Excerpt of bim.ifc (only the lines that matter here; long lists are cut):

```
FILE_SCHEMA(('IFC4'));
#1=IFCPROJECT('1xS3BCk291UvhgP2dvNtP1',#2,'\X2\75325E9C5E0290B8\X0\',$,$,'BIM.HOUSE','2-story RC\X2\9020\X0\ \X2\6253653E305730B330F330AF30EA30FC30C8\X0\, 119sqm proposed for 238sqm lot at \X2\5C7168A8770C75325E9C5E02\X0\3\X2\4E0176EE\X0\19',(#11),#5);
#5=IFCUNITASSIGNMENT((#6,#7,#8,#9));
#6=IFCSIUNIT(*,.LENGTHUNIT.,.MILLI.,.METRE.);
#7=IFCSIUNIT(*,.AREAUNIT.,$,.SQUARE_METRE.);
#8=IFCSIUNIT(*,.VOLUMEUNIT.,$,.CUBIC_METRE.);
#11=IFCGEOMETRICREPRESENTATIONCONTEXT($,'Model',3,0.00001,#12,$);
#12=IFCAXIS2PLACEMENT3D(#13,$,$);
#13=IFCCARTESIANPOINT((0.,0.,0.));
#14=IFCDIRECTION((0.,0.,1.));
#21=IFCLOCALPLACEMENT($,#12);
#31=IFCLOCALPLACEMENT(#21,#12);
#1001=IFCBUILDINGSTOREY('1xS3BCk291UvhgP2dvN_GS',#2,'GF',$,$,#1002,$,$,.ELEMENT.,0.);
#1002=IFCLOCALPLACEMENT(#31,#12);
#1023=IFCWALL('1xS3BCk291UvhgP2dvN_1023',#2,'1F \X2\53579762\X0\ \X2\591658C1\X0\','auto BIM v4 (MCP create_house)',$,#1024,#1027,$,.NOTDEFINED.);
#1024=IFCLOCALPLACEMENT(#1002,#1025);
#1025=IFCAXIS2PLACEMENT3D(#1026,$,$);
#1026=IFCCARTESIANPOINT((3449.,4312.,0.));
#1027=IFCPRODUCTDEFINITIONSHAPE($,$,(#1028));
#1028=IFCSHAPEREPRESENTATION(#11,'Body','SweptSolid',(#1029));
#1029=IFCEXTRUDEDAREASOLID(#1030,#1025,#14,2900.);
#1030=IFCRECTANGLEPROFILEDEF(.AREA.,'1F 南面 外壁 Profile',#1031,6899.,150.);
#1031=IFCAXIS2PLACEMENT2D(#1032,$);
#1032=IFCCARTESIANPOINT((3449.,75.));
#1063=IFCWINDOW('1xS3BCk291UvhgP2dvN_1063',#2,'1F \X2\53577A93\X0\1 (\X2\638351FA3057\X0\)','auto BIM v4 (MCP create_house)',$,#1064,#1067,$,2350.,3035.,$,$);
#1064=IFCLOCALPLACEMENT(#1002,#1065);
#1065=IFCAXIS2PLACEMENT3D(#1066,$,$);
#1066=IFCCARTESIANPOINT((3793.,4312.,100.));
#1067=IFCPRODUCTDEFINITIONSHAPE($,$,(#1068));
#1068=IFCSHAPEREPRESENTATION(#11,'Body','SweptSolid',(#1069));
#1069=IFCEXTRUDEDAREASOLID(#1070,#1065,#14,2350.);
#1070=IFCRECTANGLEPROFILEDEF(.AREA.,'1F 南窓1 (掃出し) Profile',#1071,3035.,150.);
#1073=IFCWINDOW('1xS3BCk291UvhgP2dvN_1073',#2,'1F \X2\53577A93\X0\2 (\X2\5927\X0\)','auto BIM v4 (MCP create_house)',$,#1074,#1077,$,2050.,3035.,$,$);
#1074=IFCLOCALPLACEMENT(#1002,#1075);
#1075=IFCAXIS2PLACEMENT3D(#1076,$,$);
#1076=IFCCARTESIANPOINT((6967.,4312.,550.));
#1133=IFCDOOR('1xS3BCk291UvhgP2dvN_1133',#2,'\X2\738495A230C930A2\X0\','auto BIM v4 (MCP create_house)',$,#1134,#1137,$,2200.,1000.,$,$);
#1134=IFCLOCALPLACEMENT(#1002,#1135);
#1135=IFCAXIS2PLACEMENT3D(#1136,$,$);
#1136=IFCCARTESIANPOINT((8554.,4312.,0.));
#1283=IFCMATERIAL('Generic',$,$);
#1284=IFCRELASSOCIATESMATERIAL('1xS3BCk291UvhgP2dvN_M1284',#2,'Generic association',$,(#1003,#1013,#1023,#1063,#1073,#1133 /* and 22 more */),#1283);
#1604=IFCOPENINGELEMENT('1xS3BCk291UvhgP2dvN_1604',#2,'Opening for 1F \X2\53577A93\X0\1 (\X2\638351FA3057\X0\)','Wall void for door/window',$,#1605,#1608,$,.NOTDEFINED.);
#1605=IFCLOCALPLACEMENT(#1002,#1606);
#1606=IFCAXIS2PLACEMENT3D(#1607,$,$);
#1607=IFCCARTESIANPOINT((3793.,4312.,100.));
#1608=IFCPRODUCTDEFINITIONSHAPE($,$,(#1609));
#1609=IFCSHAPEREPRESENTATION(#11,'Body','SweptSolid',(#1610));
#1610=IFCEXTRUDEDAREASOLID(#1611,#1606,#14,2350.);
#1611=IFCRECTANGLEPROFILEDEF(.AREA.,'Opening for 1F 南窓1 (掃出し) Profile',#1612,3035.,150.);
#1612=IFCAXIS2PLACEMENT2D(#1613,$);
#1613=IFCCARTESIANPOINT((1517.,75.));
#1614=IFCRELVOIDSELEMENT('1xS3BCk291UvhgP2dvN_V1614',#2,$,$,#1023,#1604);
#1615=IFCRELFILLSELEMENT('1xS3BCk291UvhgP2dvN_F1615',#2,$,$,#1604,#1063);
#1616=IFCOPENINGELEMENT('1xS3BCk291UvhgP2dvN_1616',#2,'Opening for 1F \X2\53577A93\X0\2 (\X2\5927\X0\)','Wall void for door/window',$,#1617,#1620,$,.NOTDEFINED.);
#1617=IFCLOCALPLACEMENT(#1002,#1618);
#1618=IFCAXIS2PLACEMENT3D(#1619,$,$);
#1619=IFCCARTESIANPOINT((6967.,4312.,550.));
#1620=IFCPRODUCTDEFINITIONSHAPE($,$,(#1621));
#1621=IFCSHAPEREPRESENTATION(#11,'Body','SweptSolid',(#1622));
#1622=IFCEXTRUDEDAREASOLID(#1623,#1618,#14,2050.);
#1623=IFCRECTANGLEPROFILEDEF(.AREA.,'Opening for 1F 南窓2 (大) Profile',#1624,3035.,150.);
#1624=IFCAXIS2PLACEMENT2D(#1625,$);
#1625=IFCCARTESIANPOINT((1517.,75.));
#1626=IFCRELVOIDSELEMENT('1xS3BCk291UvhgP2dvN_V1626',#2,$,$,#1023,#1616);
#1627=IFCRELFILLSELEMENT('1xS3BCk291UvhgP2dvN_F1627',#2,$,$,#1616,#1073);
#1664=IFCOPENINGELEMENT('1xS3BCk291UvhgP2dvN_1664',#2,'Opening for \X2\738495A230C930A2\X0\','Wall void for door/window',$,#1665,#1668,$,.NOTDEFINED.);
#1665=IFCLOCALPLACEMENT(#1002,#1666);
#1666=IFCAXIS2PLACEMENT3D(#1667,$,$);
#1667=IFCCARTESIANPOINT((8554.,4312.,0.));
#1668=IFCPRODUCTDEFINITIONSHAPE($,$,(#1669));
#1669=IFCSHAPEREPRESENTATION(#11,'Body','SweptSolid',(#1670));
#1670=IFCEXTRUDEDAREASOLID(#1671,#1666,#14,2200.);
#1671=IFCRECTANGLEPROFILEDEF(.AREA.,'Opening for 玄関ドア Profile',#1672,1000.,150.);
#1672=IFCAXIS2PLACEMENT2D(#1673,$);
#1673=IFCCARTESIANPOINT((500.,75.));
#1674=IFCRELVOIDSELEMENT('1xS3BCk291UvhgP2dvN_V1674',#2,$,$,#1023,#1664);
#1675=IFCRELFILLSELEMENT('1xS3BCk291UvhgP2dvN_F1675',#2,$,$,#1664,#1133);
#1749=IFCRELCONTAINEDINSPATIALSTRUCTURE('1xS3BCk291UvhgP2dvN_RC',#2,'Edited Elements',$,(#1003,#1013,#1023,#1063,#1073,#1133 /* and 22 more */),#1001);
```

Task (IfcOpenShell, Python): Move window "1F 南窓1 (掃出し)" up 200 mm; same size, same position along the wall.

```python
import numpy as np
import ifcopenshell
import ifcopenshell.api.geometry
import ifcopenshell.util.placement
import ifcopenshell.util.unit

model = ifcopenshell.open("bim.ifc")
unit_scale = ifcopenshell.util.unit.calculate_unit_scale(model)

window = model.by_id(1063)
opening = window.FillsVoids[0].RelatingOpeningElement
dz = 0.2 / unit_scale

shift = np.array([0.0, 0.0, dz])
# The window is not placed relative to its opening, so move both.
for product in (opening, window):
    matrix = ifcopenshell.util.placement.get_local_placement(product.ObjectPlacement)
    matrix[:3, 3] += shift
    ifcopenshell.api.geometry.edit_object_placement(model, product=product, matrix=matrix, is_si=False)

print(f"moved by {dz * unit_scale:+.3f} m")

model.write("bim_edited.ifc")
```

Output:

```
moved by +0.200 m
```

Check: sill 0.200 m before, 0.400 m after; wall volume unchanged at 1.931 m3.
